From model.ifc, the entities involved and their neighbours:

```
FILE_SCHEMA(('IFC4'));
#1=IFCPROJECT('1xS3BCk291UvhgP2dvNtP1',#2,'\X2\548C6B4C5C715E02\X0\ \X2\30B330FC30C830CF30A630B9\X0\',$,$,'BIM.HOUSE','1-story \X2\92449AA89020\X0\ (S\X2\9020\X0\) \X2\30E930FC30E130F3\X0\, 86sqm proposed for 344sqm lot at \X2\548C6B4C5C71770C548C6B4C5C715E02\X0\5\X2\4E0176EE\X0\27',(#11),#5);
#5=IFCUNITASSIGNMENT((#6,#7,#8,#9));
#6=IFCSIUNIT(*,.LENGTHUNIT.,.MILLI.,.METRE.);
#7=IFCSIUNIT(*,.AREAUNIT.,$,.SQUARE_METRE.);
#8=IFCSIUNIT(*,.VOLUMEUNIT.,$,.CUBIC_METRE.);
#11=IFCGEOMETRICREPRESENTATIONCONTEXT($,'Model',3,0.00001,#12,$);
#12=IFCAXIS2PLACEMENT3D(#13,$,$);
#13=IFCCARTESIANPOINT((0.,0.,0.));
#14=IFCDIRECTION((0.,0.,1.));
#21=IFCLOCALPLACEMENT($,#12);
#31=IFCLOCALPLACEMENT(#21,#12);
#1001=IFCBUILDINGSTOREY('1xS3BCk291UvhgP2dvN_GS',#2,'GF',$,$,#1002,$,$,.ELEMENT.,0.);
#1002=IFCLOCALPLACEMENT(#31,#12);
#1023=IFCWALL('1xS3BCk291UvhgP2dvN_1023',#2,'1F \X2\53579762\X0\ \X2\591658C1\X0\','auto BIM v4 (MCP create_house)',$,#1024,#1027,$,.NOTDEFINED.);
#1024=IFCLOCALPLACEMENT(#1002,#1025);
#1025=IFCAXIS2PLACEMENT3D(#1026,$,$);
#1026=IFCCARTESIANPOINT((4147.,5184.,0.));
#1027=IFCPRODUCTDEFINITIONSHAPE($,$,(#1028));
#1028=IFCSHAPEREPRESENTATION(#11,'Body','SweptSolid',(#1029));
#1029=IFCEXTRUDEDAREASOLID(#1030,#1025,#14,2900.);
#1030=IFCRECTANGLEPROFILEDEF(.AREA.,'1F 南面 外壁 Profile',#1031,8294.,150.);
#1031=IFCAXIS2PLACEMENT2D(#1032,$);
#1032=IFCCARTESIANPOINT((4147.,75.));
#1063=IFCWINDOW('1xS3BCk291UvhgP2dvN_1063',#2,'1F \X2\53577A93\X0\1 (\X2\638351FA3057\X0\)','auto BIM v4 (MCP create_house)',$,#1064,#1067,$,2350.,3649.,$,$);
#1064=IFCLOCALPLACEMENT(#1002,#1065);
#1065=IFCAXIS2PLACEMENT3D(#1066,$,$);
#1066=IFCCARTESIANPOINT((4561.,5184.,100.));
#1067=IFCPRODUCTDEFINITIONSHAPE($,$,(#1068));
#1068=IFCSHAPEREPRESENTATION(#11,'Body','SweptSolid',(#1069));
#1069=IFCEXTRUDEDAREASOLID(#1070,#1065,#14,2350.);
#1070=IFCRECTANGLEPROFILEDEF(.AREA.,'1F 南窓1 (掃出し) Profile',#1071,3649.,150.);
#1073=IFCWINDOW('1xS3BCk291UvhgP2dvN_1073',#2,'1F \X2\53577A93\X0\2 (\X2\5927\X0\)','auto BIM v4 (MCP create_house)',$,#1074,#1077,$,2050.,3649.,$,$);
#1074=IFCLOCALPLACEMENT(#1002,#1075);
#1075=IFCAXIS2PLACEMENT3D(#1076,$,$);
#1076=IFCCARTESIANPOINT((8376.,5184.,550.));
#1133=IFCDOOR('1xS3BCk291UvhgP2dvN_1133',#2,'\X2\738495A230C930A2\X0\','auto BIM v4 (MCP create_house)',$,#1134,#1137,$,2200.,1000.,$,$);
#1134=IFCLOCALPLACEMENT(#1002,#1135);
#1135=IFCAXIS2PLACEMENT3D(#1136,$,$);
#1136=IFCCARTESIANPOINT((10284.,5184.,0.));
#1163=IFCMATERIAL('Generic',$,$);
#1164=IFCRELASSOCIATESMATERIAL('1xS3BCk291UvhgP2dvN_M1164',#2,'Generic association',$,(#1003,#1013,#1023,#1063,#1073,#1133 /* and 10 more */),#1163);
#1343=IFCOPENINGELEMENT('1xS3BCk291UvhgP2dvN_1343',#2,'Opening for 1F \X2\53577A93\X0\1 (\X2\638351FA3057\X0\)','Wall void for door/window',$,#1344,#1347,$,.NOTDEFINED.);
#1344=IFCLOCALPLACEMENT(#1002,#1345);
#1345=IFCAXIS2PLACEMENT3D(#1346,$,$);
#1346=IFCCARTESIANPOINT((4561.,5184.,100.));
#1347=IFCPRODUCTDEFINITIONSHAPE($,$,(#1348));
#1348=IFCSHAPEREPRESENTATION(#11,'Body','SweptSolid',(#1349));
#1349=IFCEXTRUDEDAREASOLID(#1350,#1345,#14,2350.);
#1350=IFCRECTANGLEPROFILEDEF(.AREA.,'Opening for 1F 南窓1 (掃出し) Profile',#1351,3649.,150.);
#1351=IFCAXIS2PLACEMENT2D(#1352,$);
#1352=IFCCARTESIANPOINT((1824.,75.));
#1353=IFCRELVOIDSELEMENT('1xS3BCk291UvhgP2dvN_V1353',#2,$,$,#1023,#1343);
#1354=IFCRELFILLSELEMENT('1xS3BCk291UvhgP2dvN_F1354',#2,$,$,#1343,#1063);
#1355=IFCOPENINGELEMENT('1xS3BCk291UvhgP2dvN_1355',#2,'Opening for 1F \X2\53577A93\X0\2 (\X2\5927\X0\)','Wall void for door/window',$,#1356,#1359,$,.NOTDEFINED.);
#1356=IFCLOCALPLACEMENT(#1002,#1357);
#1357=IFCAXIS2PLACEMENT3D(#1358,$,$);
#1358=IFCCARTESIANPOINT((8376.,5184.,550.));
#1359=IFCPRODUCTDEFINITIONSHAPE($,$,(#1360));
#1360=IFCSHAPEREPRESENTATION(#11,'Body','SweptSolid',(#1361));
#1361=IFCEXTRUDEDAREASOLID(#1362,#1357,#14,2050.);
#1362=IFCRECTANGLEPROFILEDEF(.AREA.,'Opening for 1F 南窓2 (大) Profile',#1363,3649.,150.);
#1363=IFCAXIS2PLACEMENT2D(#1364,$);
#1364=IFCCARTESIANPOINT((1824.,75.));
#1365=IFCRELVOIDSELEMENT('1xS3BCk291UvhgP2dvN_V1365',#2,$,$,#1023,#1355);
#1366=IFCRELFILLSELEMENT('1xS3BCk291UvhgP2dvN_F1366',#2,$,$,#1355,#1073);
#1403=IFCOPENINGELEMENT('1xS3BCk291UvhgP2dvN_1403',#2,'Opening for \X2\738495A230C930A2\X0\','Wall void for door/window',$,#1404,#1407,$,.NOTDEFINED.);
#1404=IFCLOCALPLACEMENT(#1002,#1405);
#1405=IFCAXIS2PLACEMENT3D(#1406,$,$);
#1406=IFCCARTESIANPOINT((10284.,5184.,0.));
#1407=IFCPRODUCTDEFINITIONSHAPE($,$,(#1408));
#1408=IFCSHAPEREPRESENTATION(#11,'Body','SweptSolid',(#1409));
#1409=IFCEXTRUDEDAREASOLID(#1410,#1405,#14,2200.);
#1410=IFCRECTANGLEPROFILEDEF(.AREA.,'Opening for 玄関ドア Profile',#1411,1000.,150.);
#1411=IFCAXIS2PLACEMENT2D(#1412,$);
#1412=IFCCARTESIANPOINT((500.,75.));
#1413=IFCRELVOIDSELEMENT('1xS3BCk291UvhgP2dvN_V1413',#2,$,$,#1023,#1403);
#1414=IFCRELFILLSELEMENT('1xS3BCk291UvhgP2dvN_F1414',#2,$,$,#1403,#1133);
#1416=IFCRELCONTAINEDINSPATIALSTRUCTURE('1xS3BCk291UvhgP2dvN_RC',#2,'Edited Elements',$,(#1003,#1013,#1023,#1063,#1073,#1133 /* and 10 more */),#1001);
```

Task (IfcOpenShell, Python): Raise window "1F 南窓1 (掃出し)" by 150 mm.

```python
import numpy as np
import ifcopenshell
import ifcopenshell.api.geometry
import ifcopenshell.util.placement
import ifcopenshell.util.unit

model = ifcopenshell.open("model.ifc")
unit_scale = ifcopenshell.util.unit.calculate_unit_scale(model)

window = model.by_guid("1xS3BCk291UvhgP2dvN_1063")
opening = window.FillsVoids[0].RelatingOpeningElement
dz = 0.15 / unit_scale

shift = np.array([0.0, 0.0, dz])
# The window is not placed relative to its opening, so move both.
for product in (opening, window):
    matrix = ifcopenshell.util.placement.get_local_placement(product.ObjectPlacement)
    matrix[:3, 3] += shift
    ifcopenshell.api.geometry.edit_object_placement(model, product=product, matrix=matrix, is_si=False)

print(f"moved by {dz * unit_scale:+.3f} m")

model.write("model-out.ifc")
```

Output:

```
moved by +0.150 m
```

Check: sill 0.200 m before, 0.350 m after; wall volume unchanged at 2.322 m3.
